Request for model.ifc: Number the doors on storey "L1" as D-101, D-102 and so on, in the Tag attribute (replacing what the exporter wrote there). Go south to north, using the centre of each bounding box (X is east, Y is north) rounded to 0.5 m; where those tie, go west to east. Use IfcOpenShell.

First a look at what the model holds.

```python
import ifcopenshell
import ifcopenshell.util.element
import ifcopenshell.util.placement

model = ifcopenshell.open("model.ifc")
print(model.schema)
storey = next(s for s in model.by_type("IfcBuildingStorey") if s.Name == "L1")
doors = [e for e in ifcopenshell.util.element.get_decomposition(storey) if e.is_a("IfcDoor")]
for e in sorted(doors, key=lambda e: e.id()):
    origin = ifcopenshell.util.placement.get_local_placement(e.ObjectPlacement)[:3, 3]
    print(e.id(), e.Tag, e.Name, origin.round(2) + 0.0, sep=" | ")
```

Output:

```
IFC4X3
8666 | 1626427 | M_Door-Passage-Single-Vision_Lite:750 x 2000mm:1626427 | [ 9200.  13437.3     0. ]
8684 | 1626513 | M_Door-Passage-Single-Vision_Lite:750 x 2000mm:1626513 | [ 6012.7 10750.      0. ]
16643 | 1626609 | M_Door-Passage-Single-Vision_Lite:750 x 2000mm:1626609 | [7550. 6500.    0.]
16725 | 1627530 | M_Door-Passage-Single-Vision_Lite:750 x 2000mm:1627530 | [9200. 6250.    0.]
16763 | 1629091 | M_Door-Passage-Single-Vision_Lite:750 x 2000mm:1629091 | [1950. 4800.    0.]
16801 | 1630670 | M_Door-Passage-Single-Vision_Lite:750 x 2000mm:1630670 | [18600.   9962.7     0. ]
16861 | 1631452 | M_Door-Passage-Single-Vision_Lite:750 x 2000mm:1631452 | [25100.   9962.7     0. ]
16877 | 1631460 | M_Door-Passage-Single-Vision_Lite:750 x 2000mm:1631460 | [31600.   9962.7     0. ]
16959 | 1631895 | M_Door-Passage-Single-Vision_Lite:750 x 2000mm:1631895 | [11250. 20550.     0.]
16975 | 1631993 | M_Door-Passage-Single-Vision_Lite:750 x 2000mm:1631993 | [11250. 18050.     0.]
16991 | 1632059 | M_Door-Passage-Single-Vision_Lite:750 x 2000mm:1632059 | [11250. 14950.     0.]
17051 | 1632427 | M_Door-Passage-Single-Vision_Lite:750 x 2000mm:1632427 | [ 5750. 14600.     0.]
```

```python
import ifcopenshell
import ifcopenshell.geom
import ifcopenshell.util.element
import ifcopenshell.util.shape

model = ifcopenshell.open("model.ifc")
settings = ifcopenshell.geom.settings()
settings.set("use-world-coords", True)


def centre(element):
    shape = ifcopenshell.geom.create_shape(settings, element)
    return ifcopenshell.util.shape.get_bbox_centroid(shape.geometry)


storey = next(s for s in model.by_type("IfcBuildingStorey") if s.Name == "L1")
doors = [e for e in ifcopenshell.util.element.get_decomposition(storey) if e.is_a("IfcDoor")]

# Insertion points can sit at a corner or the storey origin, so sort by the geometry (in metres).
centres = {e: centre(e) for e in doors}
doors.sort(key=lambda e: (round(centres[e][1] / 0.5), centres[e][0]))

for i, e in enumerate(doors, start=1):
    number = f"D-1{i:02d}"
    e.Tag = number
    print(e.id(), number)

model.write("model_updated.ifc")
```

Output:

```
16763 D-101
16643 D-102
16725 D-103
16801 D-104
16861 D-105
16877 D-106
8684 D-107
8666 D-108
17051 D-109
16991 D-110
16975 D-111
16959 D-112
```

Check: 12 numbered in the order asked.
